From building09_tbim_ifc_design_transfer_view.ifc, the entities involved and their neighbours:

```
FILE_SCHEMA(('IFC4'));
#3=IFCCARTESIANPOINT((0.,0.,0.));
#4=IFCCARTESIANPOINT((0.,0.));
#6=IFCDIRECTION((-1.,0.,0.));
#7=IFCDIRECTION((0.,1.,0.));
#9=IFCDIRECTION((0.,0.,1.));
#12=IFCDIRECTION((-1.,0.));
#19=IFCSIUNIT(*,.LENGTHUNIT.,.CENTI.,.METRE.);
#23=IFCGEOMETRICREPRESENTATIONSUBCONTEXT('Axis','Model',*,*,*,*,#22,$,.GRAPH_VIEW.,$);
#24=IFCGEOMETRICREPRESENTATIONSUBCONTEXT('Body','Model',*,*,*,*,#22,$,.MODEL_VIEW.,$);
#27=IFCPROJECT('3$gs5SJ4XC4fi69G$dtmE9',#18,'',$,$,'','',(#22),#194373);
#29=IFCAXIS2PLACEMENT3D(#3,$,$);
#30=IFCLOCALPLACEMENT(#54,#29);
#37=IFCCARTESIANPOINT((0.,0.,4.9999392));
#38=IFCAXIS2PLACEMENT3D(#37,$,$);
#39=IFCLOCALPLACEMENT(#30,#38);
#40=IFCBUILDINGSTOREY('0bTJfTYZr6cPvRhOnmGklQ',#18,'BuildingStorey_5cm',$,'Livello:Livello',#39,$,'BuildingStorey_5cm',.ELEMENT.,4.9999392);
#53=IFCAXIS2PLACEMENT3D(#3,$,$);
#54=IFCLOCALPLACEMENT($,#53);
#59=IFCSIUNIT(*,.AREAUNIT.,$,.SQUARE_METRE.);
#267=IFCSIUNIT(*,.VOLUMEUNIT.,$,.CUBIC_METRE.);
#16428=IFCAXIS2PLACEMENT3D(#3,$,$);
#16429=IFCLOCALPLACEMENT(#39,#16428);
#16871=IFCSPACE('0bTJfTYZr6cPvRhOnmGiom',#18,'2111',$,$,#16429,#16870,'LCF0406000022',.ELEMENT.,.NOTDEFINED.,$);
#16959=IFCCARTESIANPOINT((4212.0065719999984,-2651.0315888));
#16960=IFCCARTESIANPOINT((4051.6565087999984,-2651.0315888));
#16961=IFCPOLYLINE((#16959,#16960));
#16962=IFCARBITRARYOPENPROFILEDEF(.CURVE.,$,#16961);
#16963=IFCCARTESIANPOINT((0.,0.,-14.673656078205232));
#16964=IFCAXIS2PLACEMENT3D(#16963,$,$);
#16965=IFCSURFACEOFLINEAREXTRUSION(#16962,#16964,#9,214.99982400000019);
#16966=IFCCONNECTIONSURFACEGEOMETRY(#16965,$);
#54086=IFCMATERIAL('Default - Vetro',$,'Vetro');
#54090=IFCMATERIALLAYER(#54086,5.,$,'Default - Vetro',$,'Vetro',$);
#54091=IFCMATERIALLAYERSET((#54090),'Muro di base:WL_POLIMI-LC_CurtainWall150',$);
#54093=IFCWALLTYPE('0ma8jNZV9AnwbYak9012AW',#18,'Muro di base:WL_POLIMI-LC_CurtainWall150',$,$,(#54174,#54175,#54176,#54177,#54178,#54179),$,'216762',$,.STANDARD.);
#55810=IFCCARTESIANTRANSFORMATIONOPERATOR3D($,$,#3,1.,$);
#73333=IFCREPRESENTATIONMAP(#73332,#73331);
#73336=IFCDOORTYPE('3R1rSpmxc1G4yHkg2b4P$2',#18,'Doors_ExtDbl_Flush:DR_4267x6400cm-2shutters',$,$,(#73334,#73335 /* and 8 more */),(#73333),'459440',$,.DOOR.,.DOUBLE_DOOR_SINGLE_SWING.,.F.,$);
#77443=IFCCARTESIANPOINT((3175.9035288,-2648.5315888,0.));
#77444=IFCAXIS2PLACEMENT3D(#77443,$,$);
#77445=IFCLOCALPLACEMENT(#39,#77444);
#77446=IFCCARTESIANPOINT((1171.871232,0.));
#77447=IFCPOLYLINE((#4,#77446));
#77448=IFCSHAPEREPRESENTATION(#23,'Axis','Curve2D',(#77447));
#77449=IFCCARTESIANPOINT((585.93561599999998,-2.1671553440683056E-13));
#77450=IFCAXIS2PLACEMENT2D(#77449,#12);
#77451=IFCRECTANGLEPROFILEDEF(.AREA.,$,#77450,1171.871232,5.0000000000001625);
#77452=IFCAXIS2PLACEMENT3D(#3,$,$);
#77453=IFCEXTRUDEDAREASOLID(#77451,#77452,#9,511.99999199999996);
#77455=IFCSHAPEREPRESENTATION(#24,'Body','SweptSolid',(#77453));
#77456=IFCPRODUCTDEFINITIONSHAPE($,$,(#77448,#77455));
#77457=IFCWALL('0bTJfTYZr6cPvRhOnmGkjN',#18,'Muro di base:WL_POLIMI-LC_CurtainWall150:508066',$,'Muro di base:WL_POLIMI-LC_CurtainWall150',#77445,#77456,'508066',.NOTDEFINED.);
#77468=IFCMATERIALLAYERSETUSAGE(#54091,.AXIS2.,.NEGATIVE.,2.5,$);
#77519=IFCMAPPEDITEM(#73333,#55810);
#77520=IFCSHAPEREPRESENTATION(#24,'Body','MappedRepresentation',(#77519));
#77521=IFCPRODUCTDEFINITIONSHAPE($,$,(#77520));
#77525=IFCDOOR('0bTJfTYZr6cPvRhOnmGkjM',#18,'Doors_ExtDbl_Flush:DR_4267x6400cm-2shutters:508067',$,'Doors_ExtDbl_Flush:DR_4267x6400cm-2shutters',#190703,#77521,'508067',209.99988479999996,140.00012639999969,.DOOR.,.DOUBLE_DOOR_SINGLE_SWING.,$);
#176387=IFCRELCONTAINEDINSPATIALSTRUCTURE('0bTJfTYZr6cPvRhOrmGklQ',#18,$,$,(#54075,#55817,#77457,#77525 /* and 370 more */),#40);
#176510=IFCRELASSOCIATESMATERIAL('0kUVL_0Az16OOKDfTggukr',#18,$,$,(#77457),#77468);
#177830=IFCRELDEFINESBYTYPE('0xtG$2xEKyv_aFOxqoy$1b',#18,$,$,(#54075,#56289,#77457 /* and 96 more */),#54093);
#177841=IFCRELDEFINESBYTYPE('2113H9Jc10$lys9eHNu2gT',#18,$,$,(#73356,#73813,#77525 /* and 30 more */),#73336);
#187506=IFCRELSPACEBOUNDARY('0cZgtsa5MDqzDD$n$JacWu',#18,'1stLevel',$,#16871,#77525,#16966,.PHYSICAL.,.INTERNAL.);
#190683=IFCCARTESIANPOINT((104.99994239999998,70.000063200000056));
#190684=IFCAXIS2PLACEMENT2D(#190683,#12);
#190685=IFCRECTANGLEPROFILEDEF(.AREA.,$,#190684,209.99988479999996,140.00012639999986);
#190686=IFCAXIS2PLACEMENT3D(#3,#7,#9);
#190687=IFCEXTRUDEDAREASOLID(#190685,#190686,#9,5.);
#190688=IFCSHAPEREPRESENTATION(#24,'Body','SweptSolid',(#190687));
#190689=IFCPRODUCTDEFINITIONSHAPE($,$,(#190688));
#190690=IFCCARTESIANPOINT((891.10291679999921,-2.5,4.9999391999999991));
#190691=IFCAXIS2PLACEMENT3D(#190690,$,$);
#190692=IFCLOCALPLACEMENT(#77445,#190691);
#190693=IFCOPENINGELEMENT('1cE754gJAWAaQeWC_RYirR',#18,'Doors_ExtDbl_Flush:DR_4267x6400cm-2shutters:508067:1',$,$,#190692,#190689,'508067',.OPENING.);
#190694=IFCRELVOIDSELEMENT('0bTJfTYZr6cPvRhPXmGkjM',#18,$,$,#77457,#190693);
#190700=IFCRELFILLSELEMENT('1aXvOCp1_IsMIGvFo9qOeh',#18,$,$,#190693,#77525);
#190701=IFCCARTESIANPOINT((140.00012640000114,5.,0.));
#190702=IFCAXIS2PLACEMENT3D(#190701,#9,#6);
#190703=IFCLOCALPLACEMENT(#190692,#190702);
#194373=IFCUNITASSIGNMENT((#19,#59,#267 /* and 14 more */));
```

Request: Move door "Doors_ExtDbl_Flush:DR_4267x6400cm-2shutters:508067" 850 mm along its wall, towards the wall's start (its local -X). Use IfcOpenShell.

```python
import numpy as np
import ifcopenshell
import ifcopenshell.api.geometry
import ifcopenshell.util.placement
import ifcopenshell.util.unit

model = ifcopenshell.open("building09_tbim_ifc_design_transfer_view.ifc")
unit_scale = ifcopenshell.util.unit.calculate_unit_scale(model)

door = model.by_id(77525)
opening = door.FillsVoids[0].RelatingOpeningElement
wall = opening.VoidsElements[0].RelatingBuildingElement

wall_matrix = ifcopenshell.util.placement.get_local_placement(wall.ObjectPlacement)
shift = wall_matrix[:3, 0] * -0.85 / unit_scale
before = ifcopenshell.util.placement.get_local_placement(door.ObjectPlacement)[:3, 3].copy()

# The door is placed relative to its opening, so it follows when the opening moves.
matrix = ifcopenshell.util.placement.get_local_placement(opening.ObjectPlacement)
matrix[:3, 3] += shift
ifcopenshell.api.geometry.edit_object_placement(
    model, product=opening, matrix=matrix, is_si=False, should_transform_children=True
)

# Space boundary surfaces are stored in each space's coordinates; move them too.
for rel in door.ProvidesBoundaries:
    if not rel.ConnectionGeometry:
        continue
    surface = rel.ConnectionGeometry.SurfaceOnRelatingElement
    space_matrix = ifcopenshell.util.placement.get_local_placement(rel.RelatingSpace.ObjectPlacement)
    point = np.array(surface.Position.Location.Coordinates) + space_matrix[:3, :3].T @ shift
    surface.Position = model.createIfcAxis2Placement3D(
        model.createIfcCartesianPoint(point.tolist()), surface.Position.Axis, surface.Position.RefDirection
    )

after = ifcopenshell.util.placement.get_local_placement(door.ObjectPlacement)[:3, 3]
print("door moved by", (after - before).round(3) + 0.0)

model.write("building09_tbim_ifc_design_transfer_view_edited.ifc")
```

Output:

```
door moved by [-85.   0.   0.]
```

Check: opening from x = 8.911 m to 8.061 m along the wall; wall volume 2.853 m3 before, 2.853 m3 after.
